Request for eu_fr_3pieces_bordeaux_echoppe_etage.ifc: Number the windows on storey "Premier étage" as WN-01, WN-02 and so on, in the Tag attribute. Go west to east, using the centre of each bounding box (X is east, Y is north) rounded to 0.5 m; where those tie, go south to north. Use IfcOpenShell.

First a look at what the model holds.

```python
import ifcopenshell
import ifcopenshell.util.element
import ifcopenshell.util.placement

model = ifcopenshell.open("eu_fr_3pieces_bordeaux_echoppe_etage.ifc")
print(model.schema)
storey = next(s for s in model.by_type("IfcBuildingStorey") if s.Name == "Premier étage")
windows = [e for e in ifcopenshell.util.element.get_decomposition(storey) if e.is_a("IfcWindow")]
for e in sorted(windows, key=lambda e: e.id()):
    origin = ifcopenshell.util.placement.get_local_placement(e.ObjectPlacement)[:3, 3]
    print(e.id(), e.Tag, e.Name, origin.round(2) + 0.0, sep=" | ")
```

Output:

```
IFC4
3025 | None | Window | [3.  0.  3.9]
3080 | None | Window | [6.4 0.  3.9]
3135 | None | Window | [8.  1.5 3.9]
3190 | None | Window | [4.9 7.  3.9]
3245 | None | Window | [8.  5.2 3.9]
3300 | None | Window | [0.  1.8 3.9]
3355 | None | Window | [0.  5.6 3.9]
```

```python
import ifcopenshell
import ifcopenshell.geom
import ifcopenshell.util.element
import ifcopenshell.util.shape

model = ifcopenshell.open("eu_fr_3pieces_bordeaux_echoppe_etage.ifc")
settings = ifcopenshell.geom.settings()
settings.set("use-world-coords", True)


def centre(element):
    shape = ifcopenshell.geom.create_shape(settings, element)
    return ifcopenshell.util.shape.get_bbox_centroid(shape.geometry)


storey = next(s for s in model.by_type("IfcBuildingStorey") if s.Name == "Premier étage")
windows = [e for e in ifcopenshell.util.element.get_decomposition(storey) if e.is_a("IfcWindow")]

# Insertion points can sit at a corner or the storey origin, so sort by the geometry (in metres).
centres = {e: centre(e) for e in windows}
windows.sort(key=lambda e: (round(centres[e][0] / 0.5), centres[e][1]))

for i, e in enumerate(windows, start=1):
    number = f"WN-{i:02d}"
    e.Tag = number
    print(e.id(), number)

model.write("eu_fr_3pieces_bordeaux_echoppe_etage_updated.ifc")
```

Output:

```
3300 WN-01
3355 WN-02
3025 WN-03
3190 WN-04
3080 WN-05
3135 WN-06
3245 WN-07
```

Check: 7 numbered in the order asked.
